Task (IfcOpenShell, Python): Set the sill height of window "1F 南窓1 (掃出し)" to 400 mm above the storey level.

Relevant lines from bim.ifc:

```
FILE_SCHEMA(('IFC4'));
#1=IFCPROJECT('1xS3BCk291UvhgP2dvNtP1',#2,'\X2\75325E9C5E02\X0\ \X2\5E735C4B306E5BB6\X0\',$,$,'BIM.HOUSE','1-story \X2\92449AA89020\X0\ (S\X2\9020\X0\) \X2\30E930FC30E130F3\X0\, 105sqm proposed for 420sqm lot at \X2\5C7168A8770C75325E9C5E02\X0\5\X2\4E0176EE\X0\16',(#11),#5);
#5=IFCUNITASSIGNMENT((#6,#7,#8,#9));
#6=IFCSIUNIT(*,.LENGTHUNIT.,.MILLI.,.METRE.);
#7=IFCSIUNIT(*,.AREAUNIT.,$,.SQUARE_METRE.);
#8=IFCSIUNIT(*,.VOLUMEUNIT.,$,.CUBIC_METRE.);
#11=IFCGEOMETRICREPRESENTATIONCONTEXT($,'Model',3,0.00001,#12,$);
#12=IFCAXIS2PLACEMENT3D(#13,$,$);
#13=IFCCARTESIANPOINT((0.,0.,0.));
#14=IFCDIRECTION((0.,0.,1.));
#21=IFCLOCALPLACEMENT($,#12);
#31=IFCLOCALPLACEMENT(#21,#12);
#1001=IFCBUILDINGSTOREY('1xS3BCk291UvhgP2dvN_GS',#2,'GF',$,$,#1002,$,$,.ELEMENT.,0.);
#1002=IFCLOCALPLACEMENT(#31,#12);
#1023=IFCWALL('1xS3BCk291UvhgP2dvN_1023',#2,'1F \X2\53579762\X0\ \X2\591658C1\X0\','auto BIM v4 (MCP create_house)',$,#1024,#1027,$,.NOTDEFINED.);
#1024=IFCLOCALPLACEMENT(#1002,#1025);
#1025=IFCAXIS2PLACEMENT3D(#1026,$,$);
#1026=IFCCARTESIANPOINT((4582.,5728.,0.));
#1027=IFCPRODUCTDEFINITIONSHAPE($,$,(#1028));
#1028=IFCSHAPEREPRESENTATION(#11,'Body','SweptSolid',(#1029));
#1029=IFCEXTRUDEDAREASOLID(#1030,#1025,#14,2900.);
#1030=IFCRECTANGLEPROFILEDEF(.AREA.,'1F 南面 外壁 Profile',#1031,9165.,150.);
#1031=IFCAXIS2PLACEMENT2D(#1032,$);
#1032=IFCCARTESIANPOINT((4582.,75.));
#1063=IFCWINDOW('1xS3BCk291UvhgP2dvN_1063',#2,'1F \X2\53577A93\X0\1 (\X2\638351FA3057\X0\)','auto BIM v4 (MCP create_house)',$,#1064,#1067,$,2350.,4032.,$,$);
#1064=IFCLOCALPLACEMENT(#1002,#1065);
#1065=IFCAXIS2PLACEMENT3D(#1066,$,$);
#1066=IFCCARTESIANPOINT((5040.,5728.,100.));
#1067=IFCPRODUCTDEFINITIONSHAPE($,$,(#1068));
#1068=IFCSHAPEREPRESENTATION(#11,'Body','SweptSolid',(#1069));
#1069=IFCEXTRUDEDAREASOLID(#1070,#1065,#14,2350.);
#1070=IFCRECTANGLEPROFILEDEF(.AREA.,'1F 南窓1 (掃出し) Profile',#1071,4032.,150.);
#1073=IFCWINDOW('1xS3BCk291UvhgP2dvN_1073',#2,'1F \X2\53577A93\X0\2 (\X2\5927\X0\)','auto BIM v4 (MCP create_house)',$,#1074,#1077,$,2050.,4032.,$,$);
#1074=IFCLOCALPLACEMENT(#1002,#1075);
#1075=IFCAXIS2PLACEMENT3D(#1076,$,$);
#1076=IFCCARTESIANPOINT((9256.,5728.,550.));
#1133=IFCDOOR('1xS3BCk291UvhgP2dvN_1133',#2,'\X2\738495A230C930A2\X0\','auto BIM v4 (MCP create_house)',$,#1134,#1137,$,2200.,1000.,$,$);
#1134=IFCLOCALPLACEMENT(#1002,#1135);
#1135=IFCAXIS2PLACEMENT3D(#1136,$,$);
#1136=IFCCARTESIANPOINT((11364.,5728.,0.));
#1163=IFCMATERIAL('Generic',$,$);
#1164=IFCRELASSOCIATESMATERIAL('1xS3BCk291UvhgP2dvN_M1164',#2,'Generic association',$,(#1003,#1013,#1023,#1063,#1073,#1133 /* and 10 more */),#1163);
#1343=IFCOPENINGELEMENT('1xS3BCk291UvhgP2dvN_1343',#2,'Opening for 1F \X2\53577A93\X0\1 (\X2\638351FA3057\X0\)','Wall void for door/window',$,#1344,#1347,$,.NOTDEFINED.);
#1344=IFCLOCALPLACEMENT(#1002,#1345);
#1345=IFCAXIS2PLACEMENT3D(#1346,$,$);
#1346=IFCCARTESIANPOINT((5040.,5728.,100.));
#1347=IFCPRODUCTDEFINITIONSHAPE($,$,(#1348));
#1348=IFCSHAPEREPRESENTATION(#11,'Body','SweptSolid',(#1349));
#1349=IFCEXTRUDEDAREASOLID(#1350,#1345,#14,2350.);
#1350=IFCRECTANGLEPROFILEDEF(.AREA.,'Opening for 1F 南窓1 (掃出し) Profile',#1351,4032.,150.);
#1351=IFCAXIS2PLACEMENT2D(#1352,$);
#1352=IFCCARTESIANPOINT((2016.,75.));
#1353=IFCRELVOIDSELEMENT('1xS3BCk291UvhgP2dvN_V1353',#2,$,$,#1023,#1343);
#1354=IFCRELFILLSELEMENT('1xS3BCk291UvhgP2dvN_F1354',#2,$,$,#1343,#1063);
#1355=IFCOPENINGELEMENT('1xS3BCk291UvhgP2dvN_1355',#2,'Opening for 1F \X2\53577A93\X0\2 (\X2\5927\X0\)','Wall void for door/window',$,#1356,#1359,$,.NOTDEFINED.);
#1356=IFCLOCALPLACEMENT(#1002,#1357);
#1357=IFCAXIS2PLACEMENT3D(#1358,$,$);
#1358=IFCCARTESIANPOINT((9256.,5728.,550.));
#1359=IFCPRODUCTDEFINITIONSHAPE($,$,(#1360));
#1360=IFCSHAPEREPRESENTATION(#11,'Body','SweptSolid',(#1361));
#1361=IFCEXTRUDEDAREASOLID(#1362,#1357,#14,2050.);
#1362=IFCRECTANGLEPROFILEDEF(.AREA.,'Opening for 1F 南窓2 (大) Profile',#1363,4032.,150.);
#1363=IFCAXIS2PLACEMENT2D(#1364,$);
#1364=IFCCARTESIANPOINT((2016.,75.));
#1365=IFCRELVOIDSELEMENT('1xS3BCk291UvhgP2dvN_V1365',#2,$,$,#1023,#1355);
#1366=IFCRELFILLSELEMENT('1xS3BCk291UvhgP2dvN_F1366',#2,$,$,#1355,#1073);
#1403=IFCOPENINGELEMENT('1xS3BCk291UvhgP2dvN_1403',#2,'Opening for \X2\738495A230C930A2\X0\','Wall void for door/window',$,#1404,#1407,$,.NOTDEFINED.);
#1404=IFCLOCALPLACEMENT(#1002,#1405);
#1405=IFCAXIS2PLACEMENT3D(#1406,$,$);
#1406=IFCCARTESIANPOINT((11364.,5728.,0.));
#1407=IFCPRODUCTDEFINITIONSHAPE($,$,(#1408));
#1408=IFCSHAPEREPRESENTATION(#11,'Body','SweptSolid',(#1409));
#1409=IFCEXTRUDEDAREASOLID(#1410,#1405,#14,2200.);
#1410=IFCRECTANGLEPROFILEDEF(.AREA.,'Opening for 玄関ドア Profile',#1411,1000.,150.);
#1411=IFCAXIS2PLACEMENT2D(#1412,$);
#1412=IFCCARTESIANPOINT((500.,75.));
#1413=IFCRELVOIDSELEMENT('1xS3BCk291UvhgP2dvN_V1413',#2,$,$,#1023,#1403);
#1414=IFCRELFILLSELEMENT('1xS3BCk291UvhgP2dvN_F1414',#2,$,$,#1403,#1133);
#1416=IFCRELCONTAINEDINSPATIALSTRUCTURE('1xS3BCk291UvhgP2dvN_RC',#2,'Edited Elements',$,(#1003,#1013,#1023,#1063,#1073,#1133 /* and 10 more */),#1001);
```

```python
import numpy as np
import ifcopenshell
import ifcopenshell.api.geometry
import ifcopenshell.geom
import ifcopenshell.util.element
import ifcopenshell.util.placement
import ifcopenshell.util.shape
import ifcopenshell.util.unit

model = ifcopenshell.open("bim.ifc")
unit_scale = ifcopenshell.util.unit.calculate_unit_scale(model)

window = model.by_guid("1xS3BCk291UvhgP2dvN_1063")
opening = window.FillsVoids[0].RelatingOpeningElement
storey = ifcopenshell.util.element.get_container(window, ifc_class="IfcBuildingStorey")
level = ifcopenshell.util.placement.get_local_placement(storey.ObjectPlacement)[2, 3]

# The opening's origin need not be at the sill, so measure its lowest point.
shape = ifcopenshell.geom.create_shape(ifcopenshell.geom.settings(), opening)
bottom = ifcopenshell.util.shape.get_shape_bottom_elevation(shape, shape.geometry) / unit_scale
dz = level + 400.0 - bottom

shift = np.array([0.0, 0.0, dz])
# The window is not placed relative to its opening, so move both.
for product in (opening, window):
    matrix = ifcopenshell.util.placement.get_local_placement(product.ObjectPlacement)
    matrix[:3, 3] += shift
    ifcopenshell.api.geometry.edit_object_placement(model, product=product, matrix=matrix, is_si=False)

print(f"moved by {dz * unit_scale:+.3f} m")

model.write("bim_rev.ifc")
```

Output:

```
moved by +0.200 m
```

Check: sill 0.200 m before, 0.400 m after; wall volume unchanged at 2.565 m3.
